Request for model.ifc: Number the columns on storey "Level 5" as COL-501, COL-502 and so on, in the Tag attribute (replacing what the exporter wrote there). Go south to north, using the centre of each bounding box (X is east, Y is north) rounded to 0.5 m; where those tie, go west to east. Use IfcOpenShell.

First a look at what the model holds.

```python
import ifcopenshell
import ifcopenshell.util.element
import ifcopenshell.util.placement

model = ifcopenshell.open("model.ifc")
print(model.schema)
storey = next(s for s in model.by_type("IfcBuildingStorey") if s.Name == "Level 5")
columns = [e for e in ifcopenshell.util.element.get_decomposition(storey) if e.is_a("IfcColumn")]
for e in sorted(columns, key=lambda e: e.id()):
    origin = ifcopenshell.util.placement.get_local_placement(e.ObjectPlacement)[:3, 3]
    print(e.id(), e.Tag, e.Name, origin.round(2) + 0.0, sep=" | ")
```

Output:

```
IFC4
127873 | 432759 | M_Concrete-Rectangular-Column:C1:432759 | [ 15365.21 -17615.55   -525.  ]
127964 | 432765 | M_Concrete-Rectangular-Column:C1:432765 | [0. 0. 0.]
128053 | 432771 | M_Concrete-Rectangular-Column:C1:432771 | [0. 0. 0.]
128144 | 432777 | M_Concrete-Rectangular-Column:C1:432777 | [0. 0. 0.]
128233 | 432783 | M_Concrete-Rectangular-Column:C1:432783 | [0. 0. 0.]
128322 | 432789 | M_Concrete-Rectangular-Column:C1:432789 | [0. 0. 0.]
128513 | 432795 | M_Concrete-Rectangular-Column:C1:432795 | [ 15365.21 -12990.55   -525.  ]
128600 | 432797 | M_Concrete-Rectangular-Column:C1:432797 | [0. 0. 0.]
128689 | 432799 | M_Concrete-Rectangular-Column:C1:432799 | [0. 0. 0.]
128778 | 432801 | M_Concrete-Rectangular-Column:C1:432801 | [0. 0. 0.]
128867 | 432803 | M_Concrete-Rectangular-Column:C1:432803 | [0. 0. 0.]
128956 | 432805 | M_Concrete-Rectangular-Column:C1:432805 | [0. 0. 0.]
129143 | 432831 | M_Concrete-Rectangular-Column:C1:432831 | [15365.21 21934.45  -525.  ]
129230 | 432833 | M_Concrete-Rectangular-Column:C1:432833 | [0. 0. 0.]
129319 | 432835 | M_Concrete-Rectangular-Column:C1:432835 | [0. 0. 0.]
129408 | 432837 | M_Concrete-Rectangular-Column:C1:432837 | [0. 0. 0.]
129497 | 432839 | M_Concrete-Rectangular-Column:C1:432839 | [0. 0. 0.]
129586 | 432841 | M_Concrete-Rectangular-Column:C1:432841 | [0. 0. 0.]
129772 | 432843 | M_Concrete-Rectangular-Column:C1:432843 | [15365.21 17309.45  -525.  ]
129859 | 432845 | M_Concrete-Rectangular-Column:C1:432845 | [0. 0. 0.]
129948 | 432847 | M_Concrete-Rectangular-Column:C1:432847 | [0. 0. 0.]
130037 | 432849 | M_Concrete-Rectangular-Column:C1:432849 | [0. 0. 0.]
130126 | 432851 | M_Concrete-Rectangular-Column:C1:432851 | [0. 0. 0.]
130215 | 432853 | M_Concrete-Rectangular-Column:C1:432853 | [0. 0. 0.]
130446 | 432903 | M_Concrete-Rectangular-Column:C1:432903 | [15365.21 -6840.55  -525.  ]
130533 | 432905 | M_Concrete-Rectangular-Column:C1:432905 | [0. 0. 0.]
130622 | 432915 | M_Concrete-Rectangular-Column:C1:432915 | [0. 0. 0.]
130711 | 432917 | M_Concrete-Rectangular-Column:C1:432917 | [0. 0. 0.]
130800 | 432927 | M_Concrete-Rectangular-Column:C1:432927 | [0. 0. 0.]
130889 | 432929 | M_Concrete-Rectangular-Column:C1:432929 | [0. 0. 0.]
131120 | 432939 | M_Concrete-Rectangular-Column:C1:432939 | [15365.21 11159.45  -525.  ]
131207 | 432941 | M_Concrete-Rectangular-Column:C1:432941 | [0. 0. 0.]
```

```python
import ifcopenshell
import ifcopenshell.geom
import ifcopenshell.util.element
import ifcopenshell.util.shape

model = ifcopenshell.open("model.ifc")
settings = ifcopenshell.geom.settings()
settings.set("use-world-coords", True)


def centre(element):
    shape = ifcopenshell.geom.create_shape(settings, element)
    return ifcopenshell.util.shape.get_bbox_centroid(shape.geometry)


storey = next(s for s in model.by_type("IfcBuildingStorey") if s.Name == "Level 5")
columns = [e for e in ifcopenshell.util.element.get_decomposition(storey) if e.is_a("IfcColumn")]

# Insertion points can sit at a corner or the storey origin, so sort by the geometry (in metres).
centres = {e: centre(e) for e in columns}
columns.sort(key=lambda e: (round(centres[e][1] / 0.5), centres[e][0]))

for i, e in enumerate(columns, start=1):
    number = f"COL-5{i:02d}"
    e.Tag = number
    print(e.id(), number)

model.write("model-out.ifc")
```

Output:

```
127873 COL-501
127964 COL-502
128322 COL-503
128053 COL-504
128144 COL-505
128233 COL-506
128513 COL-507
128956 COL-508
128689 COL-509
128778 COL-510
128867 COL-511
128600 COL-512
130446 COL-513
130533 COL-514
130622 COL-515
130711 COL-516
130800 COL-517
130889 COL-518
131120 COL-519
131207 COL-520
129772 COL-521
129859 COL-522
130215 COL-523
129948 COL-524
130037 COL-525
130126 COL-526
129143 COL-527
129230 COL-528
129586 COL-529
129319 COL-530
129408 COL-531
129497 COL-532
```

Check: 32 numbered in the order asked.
